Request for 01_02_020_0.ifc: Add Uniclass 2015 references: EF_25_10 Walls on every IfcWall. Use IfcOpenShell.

First a look at what the model holds.

```python
import ifcopenshell

model = ifcopenshell.open("01_02_020_0.ifc")
print(model.schema)
print("classifications:", [c.Name for c in model.by_type("IfcClassification")])
for ifc_class in ("IfcDoor", "IfcRoof", "IfcStair", "IfcWall", "IfcWindow"):
    print(ifc_class, len(model.by_type(ifc_class)))
```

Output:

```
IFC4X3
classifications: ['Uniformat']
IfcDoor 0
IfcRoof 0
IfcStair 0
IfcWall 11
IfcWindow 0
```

```python
import ifcopenshell
import ifcopenshell.api.classification

model = ifcopenshell.open("01_02_020_0.ifc")

system = ifcopenshell.api.classification.add_classification(model, classification="Uniclass 2015")

codes = {
    "IfcWall": ("EF_25_10", "Walls"),
}
for ifc_class, (code, name) in codes.items():
    products = model.by_type(ifc_class)
    ifcopenshell.api.classification.add_reference(
        model, products=products, classification=system, identification=code, name=name
    )
    print(code, len(products))

model.write("01_02_020_0_v2.ifc")
```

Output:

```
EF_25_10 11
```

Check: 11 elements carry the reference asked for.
